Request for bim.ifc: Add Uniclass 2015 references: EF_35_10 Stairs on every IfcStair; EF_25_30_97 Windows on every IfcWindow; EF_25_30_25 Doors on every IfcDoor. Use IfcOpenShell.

First a look at what the model holds.

```python
import ifcopenshell

model = ifcopenshell.open("bim.ifc")
print(model.schema)
print("classifications:", [c.Name for c in model.by_type("IfcClassification")])
for ifc_class in ("IfcDoor", "IfcRoof", "IfcStair", "IfcWall", "IfcWindow"):
    print(ifc_class, len(model.by_type(ifc_class)))
```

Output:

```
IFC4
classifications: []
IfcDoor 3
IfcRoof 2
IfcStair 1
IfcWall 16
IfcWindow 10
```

```python
import ifcopenshell
import ifcopenshell.api.classification

model = ifcopenshell.open("bim.ifc")

system = ifcopenshell.api.classification.add_classification(model, classification="Uniclass 2015")

codes = {
    "IfcStair": ("EF_35_10", "Stairs"),
    "IfcWindow": ("EF_25_30_97", "Windows"),
    "IfcDoor": ("EF_25_30_25", "Doors"),
}
for ifc_class, (code, name) in codes.items():
    products = model.by_type(ifc_class)
    ifcopenshell.api.classification.add_reference(
        model, products=products, classification=system, identification=code, name=name
    )
    print(code, len(products))

model.write("bim_v2.ifc")
```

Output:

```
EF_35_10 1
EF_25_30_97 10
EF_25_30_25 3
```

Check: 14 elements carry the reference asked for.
